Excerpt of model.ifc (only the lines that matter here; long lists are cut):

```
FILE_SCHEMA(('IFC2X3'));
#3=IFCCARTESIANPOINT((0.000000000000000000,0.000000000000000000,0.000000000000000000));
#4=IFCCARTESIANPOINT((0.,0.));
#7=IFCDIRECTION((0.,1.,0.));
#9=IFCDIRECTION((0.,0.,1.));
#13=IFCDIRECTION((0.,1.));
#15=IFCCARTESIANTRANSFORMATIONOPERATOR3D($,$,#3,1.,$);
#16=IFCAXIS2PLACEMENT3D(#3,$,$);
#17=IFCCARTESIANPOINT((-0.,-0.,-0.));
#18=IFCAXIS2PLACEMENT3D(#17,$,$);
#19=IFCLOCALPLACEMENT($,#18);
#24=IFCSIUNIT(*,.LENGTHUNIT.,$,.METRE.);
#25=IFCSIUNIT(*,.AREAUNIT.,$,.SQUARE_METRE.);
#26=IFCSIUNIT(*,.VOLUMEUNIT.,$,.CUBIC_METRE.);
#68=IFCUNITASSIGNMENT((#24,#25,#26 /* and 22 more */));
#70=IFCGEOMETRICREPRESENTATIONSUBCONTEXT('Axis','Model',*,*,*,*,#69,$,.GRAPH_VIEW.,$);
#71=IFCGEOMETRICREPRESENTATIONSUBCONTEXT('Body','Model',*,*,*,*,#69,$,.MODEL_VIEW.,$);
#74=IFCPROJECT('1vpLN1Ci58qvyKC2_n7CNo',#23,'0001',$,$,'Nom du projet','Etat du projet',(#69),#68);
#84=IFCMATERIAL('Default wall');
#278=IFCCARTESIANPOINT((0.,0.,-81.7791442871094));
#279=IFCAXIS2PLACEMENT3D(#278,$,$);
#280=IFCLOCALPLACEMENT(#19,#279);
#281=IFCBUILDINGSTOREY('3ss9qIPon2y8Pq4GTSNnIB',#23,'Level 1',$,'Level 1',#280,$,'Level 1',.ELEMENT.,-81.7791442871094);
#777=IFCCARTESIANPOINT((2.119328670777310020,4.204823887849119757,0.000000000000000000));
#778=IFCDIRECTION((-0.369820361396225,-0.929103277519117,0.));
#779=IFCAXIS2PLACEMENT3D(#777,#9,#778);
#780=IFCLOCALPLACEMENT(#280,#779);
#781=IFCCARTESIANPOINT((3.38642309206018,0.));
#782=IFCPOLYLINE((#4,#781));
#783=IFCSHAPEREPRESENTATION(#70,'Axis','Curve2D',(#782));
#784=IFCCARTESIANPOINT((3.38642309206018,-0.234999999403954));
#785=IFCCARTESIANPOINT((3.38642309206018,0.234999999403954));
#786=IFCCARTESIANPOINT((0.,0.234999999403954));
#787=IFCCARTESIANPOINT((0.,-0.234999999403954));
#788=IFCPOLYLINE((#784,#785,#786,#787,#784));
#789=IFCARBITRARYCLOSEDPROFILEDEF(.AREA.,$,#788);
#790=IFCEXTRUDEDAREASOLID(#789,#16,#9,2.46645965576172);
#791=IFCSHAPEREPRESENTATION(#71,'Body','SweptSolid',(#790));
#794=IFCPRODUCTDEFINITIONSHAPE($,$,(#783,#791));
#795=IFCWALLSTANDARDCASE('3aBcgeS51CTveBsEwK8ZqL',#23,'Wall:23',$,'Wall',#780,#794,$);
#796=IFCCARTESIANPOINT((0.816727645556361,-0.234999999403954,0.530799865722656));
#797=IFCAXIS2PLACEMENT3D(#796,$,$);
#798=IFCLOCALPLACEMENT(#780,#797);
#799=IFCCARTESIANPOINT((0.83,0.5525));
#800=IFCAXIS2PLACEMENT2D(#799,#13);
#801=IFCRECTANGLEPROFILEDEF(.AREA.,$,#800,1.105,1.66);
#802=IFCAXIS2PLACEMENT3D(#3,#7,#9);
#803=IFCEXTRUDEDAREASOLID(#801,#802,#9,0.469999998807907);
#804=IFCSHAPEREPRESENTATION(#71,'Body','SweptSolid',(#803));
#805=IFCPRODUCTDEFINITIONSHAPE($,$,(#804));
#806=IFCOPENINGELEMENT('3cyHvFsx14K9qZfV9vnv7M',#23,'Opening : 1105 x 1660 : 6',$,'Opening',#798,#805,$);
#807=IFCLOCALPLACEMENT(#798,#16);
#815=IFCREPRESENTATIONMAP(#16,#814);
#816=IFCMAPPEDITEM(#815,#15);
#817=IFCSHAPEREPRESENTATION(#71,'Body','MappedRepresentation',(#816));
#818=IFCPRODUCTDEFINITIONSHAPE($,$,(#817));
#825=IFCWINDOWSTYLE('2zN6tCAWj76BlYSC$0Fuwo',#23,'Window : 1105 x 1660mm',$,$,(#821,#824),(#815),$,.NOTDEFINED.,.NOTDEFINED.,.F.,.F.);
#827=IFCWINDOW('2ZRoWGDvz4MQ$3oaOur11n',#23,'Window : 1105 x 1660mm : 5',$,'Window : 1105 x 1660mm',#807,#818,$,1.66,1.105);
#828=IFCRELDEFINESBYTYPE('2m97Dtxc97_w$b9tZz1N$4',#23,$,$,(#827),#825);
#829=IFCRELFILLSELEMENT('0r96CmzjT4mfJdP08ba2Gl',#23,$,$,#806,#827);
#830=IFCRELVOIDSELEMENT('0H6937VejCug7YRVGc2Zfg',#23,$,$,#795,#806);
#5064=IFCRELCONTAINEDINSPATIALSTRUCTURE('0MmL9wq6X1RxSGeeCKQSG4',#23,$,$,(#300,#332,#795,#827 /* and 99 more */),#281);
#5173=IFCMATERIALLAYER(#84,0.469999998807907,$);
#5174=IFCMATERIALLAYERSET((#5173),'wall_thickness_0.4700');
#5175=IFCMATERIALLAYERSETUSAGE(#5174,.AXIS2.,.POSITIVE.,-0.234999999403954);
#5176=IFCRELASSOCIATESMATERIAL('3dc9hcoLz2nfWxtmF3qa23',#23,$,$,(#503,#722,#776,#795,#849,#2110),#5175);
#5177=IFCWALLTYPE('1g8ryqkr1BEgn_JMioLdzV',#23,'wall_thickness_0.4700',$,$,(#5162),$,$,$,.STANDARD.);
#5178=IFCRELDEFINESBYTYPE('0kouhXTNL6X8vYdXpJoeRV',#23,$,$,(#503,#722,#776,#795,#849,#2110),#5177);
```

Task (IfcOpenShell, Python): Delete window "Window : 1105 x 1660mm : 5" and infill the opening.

```python
import ifcopenshell
import ifcopenshell.api.feature
import ifcopenshell.api.root
import ifcopenshell.geom
import ifcopenshell.util.shape

model = ifcopenshell.open("model.ifc")
settings = ifcopenshell.geom.settings()


def volume(element):
    """Net volume in cubic metres, openings subtracted."""
    shape = ifcopenshell.geom.create_shape(settings, element)
    return ifcopenshell.util.shape.get_volume(shape.geometry)


window = model.by_id(827)
opening = window.FillsVoids[0].RelatingOpeningElement
wall = opening.VoidsElements[0].RelatingBuildingElement
before = volume(wall)

ifcopenshell.api.root.remove_product(model, product=window)
ifcopenshell.api.feature.remove_feature(model, feature=opening)

after = volume(wall)

print(f"wall volume {before:.3f} -> {after:.3f} m3")

model.write("model_rev.ifc")
```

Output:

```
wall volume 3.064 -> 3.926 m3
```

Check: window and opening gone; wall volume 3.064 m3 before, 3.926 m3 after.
